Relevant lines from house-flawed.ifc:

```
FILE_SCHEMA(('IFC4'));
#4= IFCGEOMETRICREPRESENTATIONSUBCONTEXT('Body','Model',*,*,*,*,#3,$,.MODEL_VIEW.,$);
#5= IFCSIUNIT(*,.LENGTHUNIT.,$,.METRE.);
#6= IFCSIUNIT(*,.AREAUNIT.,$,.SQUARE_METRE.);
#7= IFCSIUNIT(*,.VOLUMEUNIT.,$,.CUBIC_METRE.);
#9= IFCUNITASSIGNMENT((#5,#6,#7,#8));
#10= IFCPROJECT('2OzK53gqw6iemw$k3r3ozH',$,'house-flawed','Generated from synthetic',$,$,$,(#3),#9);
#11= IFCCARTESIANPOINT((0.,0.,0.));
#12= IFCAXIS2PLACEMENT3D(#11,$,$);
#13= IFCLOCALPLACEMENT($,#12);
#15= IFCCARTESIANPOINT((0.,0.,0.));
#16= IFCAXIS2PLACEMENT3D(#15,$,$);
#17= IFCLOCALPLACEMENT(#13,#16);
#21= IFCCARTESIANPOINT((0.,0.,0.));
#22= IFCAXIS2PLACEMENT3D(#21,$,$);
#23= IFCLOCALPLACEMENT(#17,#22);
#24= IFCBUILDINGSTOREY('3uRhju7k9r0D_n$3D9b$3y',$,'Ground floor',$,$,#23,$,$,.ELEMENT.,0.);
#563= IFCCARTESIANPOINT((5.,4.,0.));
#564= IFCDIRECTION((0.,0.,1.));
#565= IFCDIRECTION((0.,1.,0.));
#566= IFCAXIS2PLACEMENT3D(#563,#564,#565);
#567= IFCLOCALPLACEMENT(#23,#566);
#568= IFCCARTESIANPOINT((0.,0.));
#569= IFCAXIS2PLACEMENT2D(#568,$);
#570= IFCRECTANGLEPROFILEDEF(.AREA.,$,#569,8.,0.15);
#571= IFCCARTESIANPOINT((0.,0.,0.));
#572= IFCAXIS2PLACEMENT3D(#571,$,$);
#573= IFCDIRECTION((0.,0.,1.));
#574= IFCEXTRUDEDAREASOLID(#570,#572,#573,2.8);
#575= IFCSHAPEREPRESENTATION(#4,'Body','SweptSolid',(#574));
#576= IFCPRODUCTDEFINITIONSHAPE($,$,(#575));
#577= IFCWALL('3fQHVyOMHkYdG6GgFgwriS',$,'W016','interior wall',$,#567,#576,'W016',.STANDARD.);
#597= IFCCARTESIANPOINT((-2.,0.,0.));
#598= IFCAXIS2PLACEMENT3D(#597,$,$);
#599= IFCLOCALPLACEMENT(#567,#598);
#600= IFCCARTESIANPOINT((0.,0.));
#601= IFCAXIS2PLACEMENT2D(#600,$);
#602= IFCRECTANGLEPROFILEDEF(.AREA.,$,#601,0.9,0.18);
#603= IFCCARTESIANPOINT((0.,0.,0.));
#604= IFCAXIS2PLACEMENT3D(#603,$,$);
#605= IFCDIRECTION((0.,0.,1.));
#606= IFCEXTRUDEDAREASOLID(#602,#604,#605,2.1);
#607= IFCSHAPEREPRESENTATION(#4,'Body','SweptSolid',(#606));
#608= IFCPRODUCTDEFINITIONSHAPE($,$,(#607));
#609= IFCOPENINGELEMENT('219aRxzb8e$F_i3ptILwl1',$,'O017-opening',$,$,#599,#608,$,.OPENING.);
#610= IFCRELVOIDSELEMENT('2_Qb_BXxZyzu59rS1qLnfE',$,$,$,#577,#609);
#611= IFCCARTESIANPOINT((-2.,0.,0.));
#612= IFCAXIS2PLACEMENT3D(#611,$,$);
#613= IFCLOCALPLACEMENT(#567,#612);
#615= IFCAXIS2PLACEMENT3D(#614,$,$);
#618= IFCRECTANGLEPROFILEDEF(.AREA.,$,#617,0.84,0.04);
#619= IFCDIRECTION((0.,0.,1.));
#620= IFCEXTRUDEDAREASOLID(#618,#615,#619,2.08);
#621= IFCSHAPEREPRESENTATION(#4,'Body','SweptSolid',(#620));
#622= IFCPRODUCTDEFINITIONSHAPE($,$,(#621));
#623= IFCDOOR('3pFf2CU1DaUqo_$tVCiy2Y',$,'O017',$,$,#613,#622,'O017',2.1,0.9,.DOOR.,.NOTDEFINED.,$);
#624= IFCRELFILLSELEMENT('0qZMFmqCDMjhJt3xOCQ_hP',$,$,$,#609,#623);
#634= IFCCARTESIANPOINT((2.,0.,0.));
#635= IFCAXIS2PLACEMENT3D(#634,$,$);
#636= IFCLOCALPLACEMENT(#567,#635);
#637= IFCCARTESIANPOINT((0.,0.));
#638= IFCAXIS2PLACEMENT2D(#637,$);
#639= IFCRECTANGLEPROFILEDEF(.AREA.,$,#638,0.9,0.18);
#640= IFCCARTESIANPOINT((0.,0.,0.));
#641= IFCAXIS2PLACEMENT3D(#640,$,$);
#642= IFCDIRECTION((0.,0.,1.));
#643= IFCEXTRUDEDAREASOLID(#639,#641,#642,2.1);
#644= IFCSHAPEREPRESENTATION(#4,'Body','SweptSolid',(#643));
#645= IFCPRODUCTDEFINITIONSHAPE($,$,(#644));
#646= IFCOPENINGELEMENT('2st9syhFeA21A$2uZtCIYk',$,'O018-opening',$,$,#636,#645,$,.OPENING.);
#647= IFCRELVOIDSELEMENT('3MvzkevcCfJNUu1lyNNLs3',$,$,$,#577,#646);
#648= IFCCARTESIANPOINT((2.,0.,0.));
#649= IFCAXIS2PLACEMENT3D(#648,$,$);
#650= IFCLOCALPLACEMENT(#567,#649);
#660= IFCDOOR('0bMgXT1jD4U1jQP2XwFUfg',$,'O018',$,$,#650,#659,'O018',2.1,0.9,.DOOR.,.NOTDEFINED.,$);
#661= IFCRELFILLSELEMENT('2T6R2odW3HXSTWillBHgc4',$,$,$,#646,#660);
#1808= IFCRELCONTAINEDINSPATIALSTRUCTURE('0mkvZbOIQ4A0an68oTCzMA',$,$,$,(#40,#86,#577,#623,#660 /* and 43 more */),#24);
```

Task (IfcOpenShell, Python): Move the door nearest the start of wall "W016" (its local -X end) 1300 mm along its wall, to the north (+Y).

```python
import ifcopenshell
import ifcopenshell.api.geometry
import ifcopenshell.util.placement

model = ifcopenshell.open("house-flawed.ifc")

door = model.by_id(623)
opening = door.FillsVoids[0].RelatingOpeningElement
wall = opening.VoidsElements[0].RelatingBuildingElement

wall_matrix = ifcopenshell.util.placement.get_local_placement(wall.ObjectPlacement)
shift = wall_matrix[:3, 0] * 1.3
before = ifcopenshell.util.placement.get_local_placement(door.ObjectPlacement)[:3, 3].copy()

# The door is not placed relative to its opening, so move both.
for product in (opening, door):
    matrix = ifcopenshell.util.placement.get_local_placement(product.ObjectPlacement)
    matrix[:3, 3] += shift
    ifcopenshell.api.geometry.edit_object_placement(model, product=product, matrix=matrix, is_si=False)

after = ifcopenshell.util.placement.get_local_placement(door.ObjectPlacement)[:3, 3]
print("door moved by", (after - before).round(3) + 0.0)

model.write("house-flawed_v2.ifc")
```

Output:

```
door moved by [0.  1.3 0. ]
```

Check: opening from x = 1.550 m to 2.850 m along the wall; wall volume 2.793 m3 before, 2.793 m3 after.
